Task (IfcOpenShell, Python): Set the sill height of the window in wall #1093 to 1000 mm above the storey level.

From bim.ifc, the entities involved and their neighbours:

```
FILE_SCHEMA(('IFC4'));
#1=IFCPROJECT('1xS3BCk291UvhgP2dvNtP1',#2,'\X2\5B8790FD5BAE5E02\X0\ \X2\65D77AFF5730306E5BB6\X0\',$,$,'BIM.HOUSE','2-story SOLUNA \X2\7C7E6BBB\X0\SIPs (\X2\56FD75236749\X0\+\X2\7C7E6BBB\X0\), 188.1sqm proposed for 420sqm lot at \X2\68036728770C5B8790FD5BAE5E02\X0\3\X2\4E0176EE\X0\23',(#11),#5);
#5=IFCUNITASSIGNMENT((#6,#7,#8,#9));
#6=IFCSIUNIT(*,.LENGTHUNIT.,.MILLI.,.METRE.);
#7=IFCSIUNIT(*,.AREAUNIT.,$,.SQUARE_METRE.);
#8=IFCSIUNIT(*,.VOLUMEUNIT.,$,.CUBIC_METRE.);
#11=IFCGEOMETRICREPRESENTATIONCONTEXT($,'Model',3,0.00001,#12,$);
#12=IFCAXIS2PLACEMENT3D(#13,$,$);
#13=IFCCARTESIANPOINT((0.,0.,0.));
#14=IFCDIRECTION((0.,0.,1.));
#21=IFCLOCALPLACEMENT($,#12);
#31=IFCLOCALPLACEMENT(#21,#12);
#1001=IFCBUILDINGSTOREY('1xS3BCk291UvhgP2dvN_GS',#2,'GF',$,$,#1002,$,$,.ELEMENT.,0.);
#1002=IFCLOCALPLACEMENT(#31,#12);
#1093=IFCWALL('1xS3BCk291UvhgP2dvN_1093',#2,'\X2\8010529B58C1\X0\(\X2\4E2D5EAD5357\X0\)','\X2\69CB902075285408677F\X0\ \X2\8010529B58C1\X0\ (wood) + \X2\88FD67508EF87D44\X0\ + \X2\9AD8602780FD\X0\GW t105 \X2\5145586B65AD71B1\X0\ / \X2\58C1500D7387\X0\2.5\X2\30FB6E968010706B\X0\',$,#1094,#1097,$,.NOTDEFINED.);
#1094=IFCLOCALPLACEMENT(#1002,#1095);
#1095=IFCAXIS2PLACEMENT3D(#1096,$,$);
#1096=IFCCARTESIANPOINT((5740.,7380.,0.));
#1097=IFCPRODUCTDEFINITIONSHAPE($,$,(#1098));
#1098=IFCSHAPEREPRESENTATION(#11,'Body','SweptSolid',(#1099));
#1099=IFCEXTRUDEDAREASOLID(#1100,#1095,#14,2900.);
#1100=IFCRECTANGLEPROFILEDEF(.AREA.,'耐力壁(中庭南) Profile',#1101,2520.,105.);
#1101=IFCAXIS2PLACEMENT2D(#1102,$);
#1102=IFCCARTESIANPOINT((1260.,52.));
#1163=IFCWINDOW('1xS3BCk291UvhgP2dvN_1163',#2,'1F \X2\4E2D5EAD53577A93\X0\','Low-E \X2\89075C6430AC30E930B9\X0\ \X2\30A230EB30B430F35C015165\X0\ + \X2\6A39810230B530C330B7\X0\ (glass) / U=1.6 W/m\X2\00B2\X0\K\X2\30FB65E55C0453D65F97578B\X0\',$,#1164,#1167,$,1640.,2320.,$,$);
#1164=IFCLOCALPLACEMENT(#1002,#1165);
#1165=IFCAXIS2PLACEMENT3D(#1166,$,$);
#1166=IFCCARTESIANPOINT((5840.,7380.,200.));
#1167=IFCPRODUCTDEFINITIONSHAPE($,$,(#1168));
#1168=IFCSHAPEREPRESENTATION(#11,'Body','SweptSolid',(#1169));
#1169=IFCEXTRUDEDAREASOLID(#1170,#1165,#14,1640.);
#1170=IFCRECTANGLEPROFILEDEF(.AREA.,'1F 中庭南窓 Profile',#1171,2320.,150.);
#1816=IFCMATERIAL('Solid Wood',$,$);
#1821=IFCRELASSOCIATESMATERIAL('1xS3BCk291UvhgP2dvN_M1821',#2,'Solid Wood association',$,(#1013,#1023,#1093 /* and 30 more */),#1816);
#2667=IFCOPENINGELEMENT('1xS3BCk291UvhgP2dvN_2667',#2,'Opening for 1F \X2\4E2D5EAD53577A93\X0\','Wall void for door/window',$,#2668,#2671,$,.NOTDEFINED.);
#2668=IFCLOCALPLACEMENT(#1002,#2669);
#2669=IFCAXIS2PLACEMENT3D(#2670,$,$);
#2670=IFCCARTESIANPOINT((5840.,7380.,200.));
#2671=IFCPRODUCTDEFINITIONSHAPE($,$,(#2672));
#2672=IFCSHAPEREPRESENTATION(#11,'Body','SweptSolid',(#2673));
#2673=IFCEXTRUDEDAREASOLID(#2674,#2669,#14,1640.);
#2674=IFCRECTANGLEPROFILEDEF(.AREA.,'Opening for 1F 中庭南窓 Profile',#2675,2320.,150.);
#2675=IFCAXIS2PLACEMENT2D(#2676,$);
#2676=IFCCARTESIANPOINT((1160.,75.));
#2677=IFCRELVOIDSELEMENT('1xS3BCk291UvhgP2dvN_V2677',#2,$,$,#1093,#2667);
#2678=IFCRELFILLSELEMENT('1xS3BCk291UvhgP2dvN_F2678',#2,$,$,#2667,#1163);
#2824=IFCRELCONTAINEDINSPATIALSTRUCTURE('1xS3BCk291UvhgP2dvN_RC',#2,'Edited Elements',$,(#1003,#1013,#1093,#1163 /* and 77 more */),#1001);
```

```python
import numpy as np
import ifcopenshell
import ifcopenshell.api.geometry
import ifcopenshell.geom
import ifcopenshell.util.element
import ifcopenshell.util.placement
import ifcopenshell.util.shape
import ifcopenshell.util.unit

model = ifcopenshell.open("bim.ifc")
unit_scale = ifcopenshell.util.unit.calculate_unit_scale(model)

window = model.by_guid("1xS3BCk291UvhgP2dvN_1163")
opening = window.FillsVoids[0].RelatingOpeningElement
storey = ifcopenshell.util.element.get_container(window, ifc_class="IfcBuildingStorey")
level = ifcopenshell.util.placement.get_local_placement(storey.ObjectPlacement)[2, 3]

# The opening's origin need not be at the sill, so measure its lowest point.
shape = ifcopenshell.geom.create_shape(ifcopenshell.geom.settings(), opening)
bottom = ifcopenshell.util.shape.get_shape_bottom_elevation(shape, shape.geometry) / unit_scale
dz = level + 1 / unit_scale - bottom

shift = np.array([0.0, 0.0, dz])
# The window is not placed relative to its opening, so move both.
for product in (opening, window):
    matrix = ifcopenshell.util.placement.get_local_placement(product.ObjectPlacement)
    matrix[:3, 3] += shift
    ifcopenshell.api.geometry.edit_object_placement(model, product=product, matrix=matrix, is_si=False)

print(f"moved by {dz * unit_scale:+.3f} m")

model.write("bim_v2.ifc")
```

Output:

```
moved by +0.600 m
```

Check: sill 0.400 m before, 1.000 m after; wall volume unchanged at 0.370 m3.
